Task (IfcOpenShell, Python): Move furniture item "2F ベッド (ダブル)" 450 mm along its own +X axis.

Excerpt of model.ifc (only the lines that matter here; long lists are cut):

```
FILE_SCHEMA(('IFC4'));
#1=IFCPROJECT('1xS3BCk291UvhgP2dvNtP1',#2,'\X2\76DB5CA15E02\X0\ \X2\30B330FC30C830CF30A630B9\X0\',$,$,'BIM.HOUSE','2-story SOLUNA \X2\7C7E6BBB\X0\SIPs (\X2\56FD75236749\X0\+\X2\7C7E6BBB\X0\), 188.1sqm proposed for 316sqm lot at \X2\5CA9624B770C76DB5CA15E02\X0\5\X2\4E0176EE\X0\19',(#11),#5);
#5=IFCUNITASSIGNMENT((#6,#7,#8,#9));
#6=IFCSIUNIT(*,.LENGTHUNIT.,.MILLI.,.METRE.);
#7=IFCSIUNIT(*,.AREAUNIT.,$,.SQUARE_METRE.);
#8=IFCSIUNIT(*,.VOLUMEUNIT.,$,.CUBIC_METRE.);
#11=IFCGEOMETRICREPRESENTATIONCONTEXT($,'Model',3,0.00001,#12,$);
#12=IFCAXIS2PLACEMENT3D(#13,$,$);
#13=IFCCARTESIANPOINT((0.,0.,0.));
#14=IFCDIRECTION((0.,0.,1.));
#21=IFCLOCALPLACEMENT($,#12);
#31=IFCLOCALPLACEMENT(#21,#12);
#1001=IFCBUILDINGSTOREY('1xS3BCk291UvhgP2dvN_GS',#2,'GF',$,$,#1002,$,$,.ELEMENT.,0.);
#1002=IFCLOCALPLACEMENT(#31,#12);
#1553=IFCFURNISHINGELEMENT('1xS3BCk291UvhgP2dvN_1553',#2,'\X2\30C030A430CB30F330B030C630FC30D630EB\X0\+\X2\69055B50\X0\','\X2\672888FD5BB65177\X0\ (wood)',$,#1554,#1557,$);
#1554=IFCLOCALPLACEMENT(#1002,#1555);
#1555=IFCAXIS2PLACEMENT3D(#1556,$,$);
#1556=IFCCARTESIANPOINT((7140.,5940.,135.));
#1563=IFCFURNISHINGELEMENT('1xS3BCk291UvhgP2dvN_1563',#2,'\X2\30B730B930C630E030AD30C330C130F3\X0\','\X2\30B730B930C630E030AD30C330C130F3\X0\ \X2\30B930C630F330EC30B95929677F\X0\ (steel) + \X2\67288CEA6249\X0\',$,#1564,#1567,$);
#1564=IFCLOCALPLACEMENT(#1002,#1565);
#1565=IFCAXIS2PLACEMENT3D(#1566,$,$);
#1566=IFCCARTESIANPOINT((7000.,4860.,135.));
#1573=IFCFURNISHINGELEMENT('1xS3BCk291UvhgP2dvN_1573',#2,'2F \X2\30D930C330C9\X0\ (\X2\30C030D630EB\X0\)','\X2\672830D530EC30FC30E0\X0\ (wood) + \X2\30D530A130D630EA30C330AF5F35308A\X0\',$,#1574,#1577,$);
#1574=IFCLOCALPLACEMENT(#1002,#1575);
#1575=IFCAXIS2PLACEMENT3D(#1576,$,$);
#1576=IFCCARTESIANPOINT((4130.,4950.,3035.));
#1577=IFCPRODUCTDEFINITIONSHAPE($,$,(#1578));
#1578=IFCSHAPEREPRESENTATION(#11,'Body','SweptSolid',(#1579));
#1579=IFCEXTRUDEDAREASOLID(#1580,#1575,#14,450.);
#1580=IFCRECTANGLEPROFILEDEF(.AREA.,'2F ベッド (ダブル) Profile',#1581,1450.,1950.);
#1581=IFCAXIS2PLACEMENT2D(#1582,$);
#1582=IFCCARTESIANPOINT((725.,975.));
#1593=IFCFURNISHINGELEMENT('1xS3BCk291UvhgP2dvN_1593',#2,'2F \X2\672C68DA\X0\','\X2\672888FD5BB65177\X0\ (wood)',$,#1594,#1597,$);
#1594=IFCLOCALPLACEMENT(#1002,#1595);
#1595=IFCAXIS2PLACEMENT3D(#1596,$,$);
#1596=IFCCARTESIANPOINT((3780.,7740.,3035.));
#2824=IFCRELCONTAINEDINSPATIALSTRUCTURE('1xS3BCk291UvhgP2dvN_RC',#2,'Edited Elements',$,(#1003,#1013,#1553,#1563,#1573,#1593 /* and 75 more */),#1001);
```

```python
import ifcopenshell
import ifcopenshell.api.geometry
import ifcopenshell.util.placement

model = ifcopenshell.open("model.ifc")

item = model.by_guid("1xS3BCk291UvhgP2dvN_1573")
matrix = ifcopenshell.util.placement.get_local_placement(item.ObjectPlacement)
matrix[:3, 3] += matrix[:3, 0] * 450.0
ifcopenshell.api.geometry.edit_object_placement(model, product=item, matrix=matrix, is_si=False)

print(ifcopenshell.util.placement.get_local_placement(item.ObjectPlacement).round(3) + 0.0)

model.write("model_v2.ifc")
```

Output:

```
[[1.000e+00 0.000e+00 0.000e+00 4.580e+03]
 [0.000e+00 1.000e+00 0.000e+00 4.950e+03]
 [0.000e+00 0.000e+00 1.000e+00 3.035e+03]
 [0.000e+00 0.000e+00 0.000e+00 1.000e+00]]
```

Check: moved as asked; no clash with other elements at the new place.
